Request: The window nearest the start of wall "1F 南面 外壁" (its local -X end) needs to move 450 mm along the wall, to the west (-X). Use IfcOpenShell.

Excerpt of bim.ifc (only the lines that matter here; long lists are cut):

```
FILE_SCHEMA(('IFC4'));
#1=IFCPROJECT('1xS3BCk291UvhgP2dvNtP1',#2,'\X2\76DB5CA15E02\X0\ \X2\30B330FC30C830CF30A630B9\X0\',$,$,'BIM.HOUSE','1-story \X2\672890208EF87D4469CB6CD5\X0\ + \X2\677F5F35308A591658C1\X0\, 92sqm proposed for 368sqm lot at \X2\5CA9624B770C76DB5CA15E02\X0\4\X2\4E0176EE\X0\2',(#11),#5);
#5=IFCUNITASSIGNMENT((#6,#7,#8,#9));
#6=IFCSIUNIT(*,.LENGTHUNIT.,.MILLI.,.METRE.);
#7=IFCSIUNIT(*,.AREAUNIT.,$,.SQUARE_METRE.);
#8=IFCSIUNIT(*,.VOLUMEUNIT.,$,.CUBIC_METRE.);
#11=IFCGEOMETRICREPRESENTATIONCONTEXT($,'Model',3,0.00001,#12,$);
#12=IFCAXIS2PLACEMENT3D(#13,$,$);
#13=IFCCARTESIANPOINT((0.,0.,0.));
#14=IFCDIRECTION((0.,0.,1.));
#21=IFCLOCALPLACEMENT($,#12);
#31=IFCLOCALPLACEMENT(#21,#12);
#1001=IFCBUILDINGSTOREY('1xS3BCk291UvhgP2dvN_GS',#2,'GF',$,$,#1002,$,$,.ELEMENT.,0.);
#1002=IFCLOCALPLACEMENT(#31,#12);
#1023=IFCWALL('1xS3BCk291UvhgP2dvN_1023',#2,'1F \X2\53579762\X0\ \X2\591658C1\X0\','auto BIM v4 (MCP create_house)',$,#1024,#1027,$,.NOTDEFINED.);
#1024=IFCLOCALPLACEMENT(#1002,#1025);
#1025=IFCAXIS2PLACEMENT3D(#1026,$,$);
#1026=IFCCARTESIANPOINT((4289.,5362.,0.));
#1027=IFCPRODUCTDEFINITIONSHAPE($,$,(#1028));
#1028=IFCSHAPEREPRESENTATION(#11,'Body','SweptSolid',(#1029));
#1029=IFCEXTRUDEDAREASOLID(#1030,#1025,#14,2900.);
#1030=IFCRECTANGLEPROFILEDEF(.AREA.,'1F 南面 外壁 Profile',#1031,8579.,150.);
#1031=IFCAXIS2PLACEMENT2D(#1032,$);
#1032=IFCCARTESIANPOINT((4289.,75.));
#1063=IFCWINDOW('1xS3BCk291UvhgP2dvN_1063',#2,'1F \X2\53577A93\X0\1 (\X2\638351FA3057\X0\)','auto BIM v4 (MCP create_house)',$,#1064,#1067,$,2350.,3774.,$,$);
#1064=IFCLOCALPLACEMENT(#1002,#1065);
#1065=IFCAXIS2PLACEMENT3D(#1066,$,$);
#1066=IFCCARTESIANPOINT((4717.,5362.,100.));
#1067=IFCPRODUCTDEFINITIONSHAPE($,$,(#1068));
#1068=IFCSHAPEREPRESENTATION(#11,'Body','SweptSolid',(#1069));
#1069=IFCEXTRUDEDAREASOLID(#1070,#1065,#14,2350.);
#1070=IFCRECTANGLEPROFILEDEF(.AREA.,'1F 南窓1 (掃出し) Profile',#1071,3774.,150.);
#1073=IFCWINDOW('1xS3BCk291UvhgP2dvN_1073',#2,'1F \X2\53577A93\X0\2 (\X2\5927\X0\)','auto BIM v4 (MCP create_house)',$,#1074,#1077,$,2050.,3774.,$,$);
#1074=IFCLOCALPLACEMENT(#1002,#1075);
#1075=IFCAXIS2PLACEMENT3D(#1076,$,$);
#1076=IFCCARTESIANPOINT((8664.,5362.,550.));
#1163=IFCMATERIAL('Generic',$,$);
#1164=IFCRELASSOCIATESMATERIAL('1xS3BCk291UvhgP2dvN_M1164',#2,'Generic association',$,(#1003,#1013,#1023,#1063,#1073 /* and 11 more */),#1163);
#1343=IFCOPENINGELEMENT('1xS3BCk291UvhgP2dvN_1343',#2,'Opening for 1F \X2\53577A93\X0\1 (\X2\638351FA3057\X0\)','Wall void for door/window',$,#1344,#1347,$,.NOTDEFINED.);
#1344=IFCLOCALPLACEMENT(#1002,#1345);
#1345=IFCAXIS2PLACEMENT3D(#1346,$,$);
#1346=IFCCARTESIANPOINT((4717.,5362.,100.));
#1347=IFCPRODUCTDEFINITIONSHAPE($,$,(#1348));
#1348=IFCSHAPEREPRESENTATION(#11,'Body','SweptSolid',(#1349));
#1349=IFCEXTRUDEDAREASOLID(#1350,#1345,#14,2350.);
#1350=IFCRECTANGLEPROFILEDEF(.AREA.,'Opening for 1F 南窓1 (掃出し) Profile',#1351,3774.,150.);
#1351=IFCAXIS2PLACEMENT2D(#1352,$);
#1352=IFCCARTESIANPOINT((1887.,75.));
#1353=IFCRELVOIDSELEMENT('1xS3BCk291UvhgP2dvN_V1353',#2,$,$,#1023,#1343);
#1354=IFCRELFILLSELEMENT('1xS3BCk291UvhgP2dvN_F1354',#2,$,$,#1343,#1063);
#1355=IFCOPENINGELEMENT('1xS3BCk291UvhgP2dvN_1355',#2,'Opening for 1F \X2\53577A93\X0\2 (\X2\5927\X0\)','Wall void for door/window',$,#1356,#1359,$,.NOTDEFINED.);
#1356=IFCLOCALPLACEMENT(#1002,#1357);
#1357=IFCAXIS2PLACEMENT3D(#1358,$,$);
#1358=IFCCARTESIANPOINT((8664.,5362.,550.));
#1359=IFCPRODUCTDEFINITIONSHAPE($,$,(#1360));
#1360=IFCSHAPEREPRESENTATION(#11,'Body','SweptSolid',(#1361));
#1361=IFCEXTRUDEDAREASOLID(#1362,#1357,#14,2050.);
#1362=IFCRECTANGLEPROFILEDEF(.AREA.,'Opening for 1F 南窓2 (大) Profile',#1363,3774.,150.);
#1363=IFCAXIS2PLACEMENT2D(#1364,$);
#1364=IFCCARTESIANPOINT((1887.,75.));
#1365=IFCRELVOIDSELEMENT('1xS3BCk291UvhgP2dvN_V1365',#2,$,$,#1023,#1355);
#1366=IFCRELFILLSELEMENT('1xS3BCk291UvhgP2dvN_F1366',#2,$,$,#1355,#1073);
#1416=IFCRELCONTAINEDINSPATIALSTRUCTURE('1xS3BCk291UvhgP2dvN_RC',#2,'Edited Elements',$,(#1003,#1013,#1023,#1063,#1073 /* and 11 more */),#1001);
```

```python
import ifcopenshell
import ifcopenshell.api.geometry
import ifcopenshell.util.placement
import ifcopenshell.util.unit

model = ifcopenshell.open("bim.ifc")
unit_scale = ifcopenshell.util.unit.calculate_unit_scale(model)

window = model.by_id(1063)
opening = window.FillsVoids[0].RelatingOpeningElement
wall = opening.VoidsElements[0].RelatingBuildingElement

wall_matrix = ifcopenshell.util.placement.get_local_placement(wall.ObjectPlacement)
shift = wall_matrix[:3, 0] * -0.45 / unit_scale
before = ifcopenshell.util.placement.get_local_placement(window.ObjectPlacement)[:3, 3].copy()

# The window is not placed relative to its opening, so move both.
for product in (opening, window):
    matrix = ifcopenshell.util.placement.get_local_placement(product.ObjectPlacement)
    matrix[:3, 3] += shift
    ifcopenshell.api.geometry.edit_object_placement(model, product=product, matrix=matrix, is_si=False)

after = ifcopenshell.util.placement.get_local_placement(window.ObjectPlacement)[:3, 3]
print("window moved by", (after - before).round(3) + 0.0)

model.write("bim_edited.ifc")
```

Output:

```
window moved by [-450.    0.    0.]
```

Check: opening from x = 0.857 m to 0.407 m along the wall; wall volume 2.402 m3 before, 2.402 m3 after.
